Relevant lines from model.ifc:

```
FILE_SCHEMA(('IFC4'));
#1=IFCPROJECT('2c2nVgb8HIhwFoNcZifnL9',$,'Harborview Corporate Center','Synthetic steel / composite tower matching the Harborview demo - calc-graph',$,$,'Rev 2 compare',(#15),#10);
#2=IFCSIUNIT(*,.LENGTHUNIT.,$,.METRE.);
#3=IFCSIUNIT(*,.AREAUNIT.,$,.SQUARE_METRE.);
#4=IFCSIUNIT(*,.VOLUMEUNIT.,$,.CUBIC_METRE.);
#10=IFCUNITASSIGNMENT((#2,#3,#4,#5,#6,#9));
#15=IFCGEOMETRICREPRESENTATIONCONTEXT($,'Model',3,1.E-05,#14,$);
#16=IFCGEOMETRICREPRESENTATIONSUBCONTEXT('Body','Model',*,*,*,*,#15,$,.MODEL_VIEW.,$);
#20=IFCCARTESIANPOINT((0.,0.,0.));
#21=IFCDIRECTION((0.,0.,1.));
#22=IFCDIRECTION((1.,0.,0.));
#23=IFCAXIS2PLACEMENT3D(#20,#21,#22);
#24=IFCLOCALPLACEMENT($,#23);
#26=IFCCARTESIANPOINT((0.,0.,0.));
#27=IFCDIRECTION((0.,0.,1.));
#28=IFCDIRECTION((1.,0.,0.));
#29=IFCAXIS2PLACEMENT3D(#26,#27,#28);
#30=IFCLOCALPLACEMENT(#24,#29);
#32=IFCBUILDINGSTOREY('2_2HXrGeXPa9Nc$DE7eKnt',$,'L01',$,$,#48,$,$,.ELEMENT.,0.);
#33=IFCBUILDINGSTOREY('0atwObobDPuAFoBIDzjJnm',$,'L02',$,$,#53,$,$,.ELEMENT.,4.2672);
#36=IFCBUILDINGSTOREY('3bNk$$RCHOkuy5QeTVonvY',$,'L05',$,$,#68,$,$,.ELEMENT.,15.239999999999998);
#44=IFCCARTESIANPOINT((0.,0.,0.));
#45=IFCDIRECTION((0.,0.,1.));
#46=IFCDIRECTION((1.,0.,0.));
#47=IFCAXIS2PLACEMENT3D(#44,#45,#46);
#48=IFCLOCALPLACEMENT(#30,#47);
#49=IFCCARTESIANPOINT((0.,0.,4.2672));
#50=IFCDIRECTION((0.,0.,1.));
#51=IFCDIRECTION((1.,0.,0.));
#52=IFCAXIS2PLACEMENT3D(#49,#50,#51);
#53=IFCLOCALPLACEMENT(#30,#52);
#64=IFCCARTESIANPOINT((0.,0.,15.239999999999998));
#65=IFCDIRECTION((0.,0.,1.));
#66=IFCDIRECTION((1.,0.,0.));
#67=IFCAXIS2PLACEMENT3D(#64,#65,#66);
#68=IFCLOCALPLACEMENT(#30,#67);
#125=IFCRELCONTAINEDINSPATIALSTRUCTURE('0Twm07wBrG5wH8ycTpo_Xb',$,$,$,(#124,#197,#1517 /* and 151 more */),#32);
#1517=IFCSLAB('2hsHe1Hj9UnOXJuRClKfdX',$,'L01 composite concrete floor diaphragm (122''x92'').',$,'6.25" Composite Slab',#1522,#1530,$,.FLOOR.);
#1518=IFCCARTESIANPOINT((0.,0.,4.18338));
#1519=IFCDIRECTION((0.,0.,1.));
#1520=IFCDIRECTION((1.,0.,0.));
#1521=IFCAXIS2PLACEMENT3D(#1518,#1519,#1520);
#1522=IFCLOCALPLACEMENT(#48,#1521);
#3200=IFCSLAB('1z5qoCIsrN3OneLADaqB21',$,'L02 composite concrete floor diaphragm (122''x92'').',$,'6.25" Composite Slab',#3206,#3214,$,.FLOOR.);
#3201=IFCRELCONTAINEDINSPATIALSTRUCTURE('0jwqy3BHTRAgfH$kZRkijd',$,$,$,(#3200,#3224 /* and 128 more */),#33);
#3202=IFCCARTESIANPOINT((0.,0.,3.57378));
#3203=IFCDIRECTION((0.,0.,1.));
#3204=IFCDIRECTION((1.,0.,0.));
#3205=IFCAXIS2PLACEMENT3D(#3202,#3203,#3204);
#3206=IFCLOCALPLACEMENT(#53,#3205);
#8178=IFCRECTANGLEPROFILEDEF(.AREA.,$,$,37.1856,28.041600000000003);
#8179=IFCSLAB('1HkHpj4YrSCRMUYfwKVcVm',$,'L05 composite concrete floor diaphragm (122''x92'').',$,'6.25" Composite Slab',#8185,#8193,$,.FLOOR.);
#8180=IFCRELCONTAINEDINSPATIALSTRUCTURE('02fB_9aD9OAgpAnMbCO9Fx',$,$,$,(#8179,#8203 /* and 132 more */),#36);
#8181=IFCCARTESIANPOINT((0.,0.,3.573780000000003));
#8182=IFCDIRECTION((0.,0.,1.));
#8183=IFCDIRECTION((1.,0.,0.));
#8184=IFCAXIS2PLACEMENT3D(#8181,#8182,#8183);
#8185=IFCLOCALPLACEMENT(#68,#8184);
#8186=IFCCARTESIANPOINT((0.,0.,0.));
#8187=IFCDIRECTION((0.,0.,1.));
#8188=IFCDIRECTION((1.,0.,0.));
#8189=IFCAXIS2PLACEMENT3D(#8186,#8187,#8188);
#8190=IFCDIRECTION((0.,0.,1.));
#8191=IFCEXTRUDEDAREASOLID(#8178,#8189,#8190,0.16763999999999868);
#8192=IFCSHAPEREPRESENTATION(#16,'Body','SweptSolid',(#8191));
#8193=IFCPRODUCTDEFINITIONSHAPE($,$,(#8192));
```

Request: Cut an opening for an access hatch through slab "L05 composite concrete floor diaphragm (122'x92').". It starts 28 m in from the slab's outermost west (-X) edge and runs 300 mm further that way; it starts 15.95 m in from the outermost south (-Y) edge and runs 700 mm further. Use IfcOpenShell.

```python
import numpy as np
import ifcopenshell
import ifcopenshell.api.feature
import ifcopenshell.api.geometry
import ifcopenshell.api.root
import ifcopenshell.geom
import ifcopenshell.util.placement
import ifcopenshell.util.representation
import ifcopenshell.util.shape
import ifcopenshell.util.unit

model = ifcopenshell.open("model.ifc")
unit_scale = ifcopenshell.util.unit.calculate_unit_scale(model)
settings = ifcopenshell.geom.settings()


def volume(element):
    """Net volume in cubic metres, openings subtracted."""
    shape = ifcopenshell.geom.create_shape(settings, element)
    return ifcopenshell.util.shape.get_volume(shape.geometry)


slab = model.by_guid("1HkHpj4YrSCRMUYfwKVcVm")
before = volume(slab)

# Extent in the slab's own axes, in metres. The edges named are its -X and -Y sides.
slab_shape = ifcopenshell.geom.create_shape(settings, slab)
vertices = ifcopenshell.util.shape.get_vertices(slab_shape.geometry)
x_min, y_min, bottom = vertices.min(axis=0)
top = vertices[:, 2].max()

opening = ifcopenshell.api.root.create_entity(model, ifc_class="IfcOpeningElement", name="Access hatch opening", predefined_type="OPENING")
context = ifcopenshell.util.representation.get_context(model, "Model", "Body", "MODEL_VIEW")
width, depth = 0.3, 0.7
outline = [(0.0, 0.0), (width, 0.0), (width, depth), (0.0, depth), (0.0, 0.0)]
# Overshoot both faces by 50 mm so the cut is clean.
shape = ifcopenshell.api.geometry.add_slab_representation(
    model, context=context, depth=top - bottom + 0.1, polyline=outline
)
ifcopenshell.api.geometry.assign_representation(model, product=opening, representation=shape)

matrix = ifcopenshell.util.placement.get_local_placement(slab.ObjectPlacement)
matrix[:, 3] = matrix @ np.append(np.array([x_min + 28, y_min + 15.95, bottom - 0.05]) / unit_scale, 1.0)
ifcopenshell.api.geometry.edit_object_placement(model, product=opening, matrix=matrix, is_si=False)
ifcopenshell.api.feature.add_feature(model, feature=opening, element=slab)

after = volume(slab)

print(f"slab volume {before:.3f} -> {after:.3f} m3")

model.write("model_rev.ifc")
```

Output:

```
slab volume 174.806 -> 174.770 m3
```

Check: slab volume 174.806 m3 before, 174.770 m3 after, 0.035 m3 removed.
